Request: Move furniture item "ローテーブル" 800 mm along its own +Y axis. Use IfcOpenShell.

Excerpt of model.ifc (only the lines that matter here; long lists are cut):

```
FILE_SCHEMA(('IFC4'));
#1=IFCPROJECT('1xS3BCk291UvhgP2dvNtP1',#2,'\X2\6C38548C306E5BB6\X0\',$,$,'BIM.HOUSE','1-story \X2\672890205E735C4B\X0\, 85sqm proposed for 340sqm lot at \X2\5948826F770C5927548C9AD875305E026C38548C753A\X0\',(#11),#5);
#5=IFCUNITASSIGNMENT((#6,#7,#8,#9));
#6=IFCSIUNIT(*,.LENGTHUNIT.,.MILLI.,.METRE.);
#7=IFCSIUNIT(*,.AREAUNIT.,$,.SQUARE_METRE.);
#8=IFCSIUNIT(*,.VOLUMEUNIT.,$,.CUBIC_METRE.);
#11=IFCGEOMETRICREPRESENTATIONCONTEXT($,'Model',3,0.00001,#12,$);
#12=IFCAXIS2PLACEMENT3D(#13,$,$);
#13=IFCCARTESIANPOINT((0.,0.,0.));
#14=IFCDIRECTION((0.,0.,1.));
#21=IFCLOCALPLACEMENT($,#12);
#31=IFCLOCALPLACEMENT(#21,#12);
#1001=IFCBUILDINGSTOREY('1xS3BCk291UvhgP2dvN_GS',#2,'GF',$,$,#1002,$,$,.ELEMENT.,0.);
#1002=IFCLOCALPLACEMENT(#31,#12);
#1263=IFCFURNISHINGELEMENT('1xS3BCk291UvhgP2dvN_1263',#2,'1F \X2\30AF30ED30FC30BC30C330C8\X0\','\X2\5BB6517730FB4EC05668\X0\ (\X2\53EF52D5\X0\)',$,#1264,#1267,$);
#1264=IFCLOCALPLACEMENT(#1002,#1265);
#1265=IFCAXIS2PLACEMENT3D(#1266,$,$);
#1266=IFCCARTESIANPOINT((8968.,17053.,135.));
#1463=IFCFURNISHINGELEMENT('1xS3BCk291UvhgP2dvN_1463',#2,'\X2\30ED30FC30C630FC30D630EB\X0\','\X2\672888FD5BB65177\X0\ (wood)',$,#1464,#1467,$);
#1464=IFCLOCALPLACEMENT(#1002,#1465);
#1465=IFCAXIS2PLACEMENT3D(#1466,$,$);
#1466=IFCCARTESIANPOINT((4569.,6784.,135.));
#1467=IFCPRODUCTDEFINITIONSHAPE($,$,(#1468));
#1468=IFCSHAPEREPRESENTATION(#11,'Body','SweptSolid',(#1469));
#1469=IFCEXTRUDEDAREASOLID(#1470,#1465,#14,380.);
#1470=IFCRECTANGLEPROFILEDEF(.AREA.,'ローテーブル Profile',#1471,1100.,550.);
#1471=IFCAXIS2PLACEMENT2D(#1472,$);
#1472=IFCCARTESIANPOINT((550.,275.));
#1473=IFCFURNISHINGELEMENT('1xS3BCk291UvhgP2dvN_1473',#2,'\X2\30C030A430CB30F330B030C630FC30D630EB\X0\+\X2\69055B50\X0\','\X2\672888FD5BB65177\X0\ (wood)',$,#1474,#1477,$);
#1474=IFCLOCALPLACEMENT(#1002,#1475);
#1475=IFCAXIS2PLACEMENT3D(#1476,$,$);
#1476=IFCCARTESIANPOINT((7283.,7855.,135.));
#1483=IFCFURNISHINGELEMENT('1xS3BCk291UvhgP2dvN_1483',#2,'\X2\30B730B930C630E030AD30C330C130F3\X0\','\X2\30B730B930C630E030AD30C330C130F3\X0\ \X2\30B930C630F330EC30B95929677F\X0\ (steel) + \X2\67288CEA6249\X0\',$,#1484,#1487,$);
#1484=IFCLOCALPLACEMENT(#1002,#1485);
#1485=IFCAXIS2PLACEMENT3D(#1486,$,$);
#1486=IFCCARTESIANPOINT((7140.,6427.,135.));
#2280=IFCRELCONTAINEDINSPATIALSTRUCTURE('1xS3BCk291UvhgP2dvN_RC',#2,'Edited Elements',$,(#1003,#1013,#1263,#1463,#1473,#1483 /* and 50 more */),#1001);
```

```python
import ifcopenshell
import ifcopenshell.api.geometry
import ifcopenshell.util.placement
import ifcopenshell.util.unit

model = ifcopenshell.open("model.ifc")
unit_scale = ifcopenshell.util.unit.calculate_unit_scale(model)

item = model.by_guid("1xS3BCk291UvhgP2dvN_1463")
matrix = ifcopenshell.util.placement.get_local_placement(item.ObjectPlacement)
matrix[:3, 3] += matrix[:3, 1] * 0.8 / unit_scale
ifcopenshell.api.geometry.edit_object_placement(model, product=item, matrix=matrix, is_si=False)

print(ifcopenshell.util.placement.get_local_placement(item.ObjectPlacement).round(3) + 0.0)

model.write("model_edited.ifc")
```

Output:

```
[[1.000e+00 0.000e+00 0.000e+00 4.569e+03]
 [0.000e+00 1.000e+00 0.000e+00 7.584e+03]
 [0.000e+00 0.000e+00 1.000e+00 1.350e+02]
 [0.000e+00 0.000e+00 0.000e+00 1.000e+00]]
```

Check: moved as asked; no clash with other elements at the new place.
